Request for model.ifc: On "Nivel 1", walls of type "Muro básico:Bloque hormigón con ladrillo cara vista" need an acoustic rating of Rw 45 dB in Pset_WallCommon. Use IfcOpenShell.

First a look at what the model holds.

```python
import ifcopenshell
import ifcopenshell.util.element

model = ifcopenshell.open("model.ifc")
print(model.schema)
storey = next(s for s in model.by_type("IfcBuildingStorey") if s.Name == "Nivel 1")
walls = [e for e in ifcopenshell.util.element.get_decomposition(storey) if e.is_a("IfcWall")]
seen = {}
for e in walls:
    element_type = ifcopenshell.util.element.get_type(e)
    key = (element_type.Name if element_type != e and element_type else None, ifcopenshell.util.element.get_pset(e, "Pset_WallCommon", "AcousticRating"))
    seen[key] = seen.get(key, 0) + 1
for (name, value), count in sorted(seen.items(), key=str):
    print(count, "x", name, "|", value)
```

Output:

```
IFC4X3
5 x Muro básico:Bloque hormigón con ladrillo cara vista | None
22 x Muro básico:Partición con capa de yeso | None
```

```python
import ifcopenshell
import ifcopenshell.api.pset
import ifcopenshell.util.element

model = ifcopenshell.open("model.ifc")

storey = next(s for s in model.by_type("IfcBuildingStorey") if s.Name == "Nivel 1")
walls = [e for e in ifcopenshell.util.element.get_decomposition(storey) if e.is_a("IfcWall")]

count = 0
for e in walls:
    element_type = ifcopenshell.util.element.get_type(e)
    if element_type in (None, e) or element_type.Name != "Muro básico:Bloque hormigón con ladrillo cara vista":
        continue
    # add_pset returns the element's existing set when there is one.
    pset = ifcopenshell.api.pset.add_pset(model, product=e, name="Pset_WallCommon")
    ifcopenshell.api.pset.edit_pset(model, pset=pset, properties={"AcousticRating": "Rw 45 dB"})
    count += 1

print(count, "walls updated")

model.write("model_edited.ifc")
```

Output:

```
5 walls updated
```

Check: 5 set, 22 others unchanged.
